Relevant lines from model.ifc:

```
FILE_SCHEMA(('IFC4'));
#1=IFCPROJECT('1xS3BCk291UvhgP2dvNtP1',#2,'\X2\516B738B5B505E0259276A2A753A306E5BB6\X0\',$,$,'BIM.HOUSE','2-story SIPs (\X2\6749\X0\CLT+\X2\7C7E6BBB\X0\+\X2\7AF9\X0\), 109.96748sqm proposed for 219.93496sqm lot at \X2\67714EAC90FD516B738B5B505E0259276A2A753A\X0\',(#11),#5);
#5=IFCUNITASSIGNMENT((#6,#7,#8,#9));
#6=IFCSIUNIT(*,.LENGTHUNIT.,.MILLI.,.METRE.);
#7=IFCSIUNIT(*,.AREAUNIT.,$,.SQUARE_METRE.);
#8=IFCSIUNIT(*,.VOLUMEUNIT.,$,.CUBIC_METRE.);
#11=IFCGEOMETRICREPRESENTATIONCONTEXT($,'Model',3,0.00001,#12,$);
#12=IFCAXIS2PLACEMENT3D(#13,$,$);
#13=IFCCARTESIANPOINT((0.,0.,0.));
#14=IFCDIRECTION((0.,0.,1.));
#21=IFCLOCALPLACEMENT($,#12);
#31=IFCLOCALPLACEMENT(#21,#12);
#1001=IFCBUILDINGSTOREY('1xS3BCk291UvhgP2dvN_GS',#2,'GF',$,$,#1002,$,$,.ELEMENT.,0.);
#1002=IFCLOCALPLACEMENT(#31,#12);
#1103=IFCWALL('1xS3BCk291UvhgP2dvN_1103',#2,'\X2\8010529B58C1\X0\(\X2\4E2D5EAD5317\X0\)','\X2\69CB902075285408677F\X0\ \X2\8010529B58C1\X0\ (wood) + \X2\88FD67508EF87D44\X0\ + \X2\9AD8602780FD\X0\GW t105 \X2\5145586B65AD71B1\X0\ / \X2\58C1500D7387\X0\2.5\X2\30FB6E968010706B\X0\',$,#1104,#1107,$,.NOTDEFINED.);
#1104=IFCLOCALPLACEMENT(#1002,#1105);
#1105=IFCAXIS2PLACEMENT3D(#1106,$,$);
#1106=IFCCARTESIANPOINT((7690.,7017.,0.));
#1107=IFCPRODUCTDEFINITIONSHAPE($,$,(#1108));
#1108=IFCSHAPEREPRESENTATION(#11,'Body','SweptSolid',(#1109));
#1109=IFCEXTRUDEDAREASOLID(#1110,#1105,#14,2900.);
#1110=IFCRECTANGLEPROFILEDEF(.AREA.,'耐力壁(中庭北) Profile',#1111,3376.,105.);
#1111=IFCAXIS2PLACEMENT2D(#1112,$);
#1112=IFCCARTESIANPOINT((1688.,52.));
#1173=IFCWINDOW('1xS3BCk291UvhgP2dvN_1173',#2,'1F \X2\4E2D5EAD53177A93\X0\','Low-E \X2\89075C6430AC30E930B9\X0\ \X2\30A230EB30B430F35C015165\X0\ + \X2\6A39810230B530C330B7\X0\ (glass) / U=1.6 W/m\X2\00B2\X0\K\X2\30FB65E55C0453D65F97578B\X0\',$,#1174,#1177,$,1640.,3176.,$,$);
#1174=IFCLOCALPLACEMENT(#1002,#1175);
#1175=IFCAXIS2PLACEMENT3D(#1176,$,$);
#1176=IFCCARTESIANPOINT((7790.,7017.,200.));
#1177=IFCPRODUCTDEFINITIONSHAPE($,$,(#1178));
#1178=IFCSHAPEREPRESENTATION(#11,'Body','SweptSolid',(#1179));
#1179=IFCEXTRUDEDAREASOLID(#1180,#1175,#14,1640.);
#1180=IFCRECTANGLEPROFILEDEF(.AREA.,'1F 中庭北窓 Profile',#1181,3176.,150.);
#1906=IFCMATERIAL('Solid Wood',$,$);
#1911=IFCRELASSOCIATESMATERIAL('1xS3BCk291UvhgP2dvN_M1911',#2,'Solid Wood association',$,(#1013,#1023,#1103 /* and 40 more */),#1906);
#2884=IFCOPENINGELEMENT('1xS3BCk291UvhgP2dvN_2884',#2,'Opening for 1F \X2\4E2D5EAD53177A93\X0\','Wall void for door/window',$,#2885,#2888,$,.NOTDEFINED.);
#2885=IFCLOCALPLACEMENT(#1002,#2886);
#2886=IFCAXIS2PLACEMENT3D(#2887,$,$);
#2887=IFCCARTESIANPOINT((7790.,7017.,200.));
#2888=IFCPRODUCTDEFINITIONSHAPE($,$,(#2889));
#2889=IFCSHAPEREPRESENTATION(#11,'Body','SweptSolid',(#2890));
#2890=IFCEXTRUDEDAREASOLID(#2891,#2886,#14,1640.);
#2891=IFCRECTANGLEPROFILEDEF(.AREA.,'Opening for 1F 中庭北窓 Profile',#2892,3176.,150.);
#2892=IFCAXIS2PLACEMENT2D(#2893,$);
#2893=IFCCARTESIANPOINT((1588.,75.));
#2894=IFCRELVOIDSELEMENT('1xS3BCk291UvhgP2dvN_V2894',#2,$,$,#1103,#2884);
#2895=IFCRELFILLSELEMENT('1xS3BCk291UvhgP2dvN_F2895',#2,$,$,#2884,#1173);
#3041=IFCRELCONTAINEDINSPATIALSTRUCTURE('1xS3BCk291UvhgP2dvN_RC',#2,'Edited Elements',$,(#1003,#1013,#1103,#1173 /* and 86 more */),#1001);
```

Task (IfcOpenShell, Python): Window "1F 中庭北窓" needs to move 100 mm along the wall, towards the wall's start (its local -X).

```python
import ifcopenshell
import ifcopenshell.api.geometry
import ifcopenshell.util.placement
import ifcopenshell.util.unit

model = ifcopenshell.open("model.ifc")
unit_scale = ifcopenshell.util.unit.calculate_unit_scale(model)

window = model.by_guid("1xS3BCk291UvhgP2dvN_1173")
opening = window.FillsVoids[0].RelatingOpeningElement
wall = opening.VoidsElements[0].RelatingBuildingElement

wall_matrix = ifcopenshell.util.placement.get_local_placement(wall.ObjectPlacement)
shift = wall_matrix[:3, 0] * -0.1 / unit_scale
before = ifcopenshell.util.placement.get_local_placement(window.ObjectPlacement)[:3, 3].copy()

# The window is not placed relative to its opening, so move both.
for product in (opening, window):
    matrix = ifcopenshell.util.placement.get_local_placement(product.ObjectPlacement)
    matrix[:3, 3] += shift
    ifcopenshell.api.geometry.edit_object_placement(model, product=product, matrix=matrix, is_si=False)

after = ifcopenshell.util.placement.get_local_placement(window.ObjectPlacement)[:3, 3]
print("window moved by", (after - before).round(3) + 0.0)

model.write("model-out.ifc")
```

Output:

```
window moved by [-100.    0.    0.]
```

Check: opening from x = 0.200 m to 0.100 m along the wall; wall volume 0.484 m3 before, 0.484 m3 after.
